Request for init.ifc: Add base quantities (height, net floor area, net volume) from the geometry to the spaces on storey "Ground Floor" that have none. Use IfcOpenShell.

First a look at what the model holds.

```python
import ifcopenshell
import ifcopenshell.util.element
import ifcopenshell.util.unit

model = ifcopenshell.open("init.ifc")
print(model.schema)
for unit_type in ("LENGTHUNIT", "AREAUNIT", "VOLUMEUNIT"):
    print(unit_type, ifcopenshell.util.unit.calculate_unit_scale(model, unit_type))
storey = next(s for s in model.by_type("IfcBuildingStorey") if s.Name == "Ground Floor")
spaces = [e for e in ifcopenshell.util.element.get_decomposition(storey) if e.is_a("IfcSpace")]
for e in sorted(spaces, key=lambda e: e.id()):
    print(e.id(), e.is_a(), e.Name, list(ifcopenshell.util.element.get_psets(e, qtos_only=True)), sep=" | ")
```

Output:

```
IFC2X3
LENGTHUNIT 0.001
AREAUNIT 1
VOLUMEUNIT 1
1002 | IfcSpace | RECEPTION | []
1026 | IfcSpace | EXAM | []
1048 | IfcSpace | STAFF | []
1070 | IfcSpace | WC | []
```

```python
import ifcopenshell
import ifcopenshell.api.pset
import ifcopenshell.geom
import ifcopenshell.util.element
import ifcopenshell.util.shape
import ifcopenshell.util.unit

model = ifcopenshell.open("init.ifc")
unit_scale = ifcopenshell.util.unit.calculate_unit_scale(model)
area_scale = ifcopenshell.util.unit.calculate_unit_scale(model, "AREAUNIT")
volume_scale = ifcopenshell.util.unit.calculate_unit_scale(model, "VOLUMEUNIT")
settings = ifcopenshell.geom.settings()

storey = next(s for s in model.by_type("IfcBuildingStorey") if s.Name == "Ground Floor")
spaces = [e for e in ifcopenshell.util.element.get_decomposition(storey) if e.is_a("IfcSpace")]

for e in sorted(spaces, key=lambda e: e.id()):
    if ifcopenshell.util.element.get_psets(e, qtos_only=True, should_inherit=False):
        continue
    # Geometry comes back in metres, in the element's own axes.
    shape = ifcopenshell.geom.create_shape(settings, e)
    values = {
        "Height": ifcopenshell.util.shape.get_z(shape.geometry) / unit_scale,
        "NetFloorArea": ifcopenshell.util.shape.get_footprint_area(shape.geometry) / area_scale,
        "NetVolume": ifcopenshell.util.shape.get_volume(shape.geometry) / volume_scale,
    }
    qto = ifcopenshell.api.pset.add_qto(model, product=e, name="BaseQuantities")
    ifcopenshell.api.pset.edit_qto(model, qto=qto, properties=values)
    print(e.id(), {k: round(v, 3) for k, v in values.items()})

model.write("init_rev.ifc")
```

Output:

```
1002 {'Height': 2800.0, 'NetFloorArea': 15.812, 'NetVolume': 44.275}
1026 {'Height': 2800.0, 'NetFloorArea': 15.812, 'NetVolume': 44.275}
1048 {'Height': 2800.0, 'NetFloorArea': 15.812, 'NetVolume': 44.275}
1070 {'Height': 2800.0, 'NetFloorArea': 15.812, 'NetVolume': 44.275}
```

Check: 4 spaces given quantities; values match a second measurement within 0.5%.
